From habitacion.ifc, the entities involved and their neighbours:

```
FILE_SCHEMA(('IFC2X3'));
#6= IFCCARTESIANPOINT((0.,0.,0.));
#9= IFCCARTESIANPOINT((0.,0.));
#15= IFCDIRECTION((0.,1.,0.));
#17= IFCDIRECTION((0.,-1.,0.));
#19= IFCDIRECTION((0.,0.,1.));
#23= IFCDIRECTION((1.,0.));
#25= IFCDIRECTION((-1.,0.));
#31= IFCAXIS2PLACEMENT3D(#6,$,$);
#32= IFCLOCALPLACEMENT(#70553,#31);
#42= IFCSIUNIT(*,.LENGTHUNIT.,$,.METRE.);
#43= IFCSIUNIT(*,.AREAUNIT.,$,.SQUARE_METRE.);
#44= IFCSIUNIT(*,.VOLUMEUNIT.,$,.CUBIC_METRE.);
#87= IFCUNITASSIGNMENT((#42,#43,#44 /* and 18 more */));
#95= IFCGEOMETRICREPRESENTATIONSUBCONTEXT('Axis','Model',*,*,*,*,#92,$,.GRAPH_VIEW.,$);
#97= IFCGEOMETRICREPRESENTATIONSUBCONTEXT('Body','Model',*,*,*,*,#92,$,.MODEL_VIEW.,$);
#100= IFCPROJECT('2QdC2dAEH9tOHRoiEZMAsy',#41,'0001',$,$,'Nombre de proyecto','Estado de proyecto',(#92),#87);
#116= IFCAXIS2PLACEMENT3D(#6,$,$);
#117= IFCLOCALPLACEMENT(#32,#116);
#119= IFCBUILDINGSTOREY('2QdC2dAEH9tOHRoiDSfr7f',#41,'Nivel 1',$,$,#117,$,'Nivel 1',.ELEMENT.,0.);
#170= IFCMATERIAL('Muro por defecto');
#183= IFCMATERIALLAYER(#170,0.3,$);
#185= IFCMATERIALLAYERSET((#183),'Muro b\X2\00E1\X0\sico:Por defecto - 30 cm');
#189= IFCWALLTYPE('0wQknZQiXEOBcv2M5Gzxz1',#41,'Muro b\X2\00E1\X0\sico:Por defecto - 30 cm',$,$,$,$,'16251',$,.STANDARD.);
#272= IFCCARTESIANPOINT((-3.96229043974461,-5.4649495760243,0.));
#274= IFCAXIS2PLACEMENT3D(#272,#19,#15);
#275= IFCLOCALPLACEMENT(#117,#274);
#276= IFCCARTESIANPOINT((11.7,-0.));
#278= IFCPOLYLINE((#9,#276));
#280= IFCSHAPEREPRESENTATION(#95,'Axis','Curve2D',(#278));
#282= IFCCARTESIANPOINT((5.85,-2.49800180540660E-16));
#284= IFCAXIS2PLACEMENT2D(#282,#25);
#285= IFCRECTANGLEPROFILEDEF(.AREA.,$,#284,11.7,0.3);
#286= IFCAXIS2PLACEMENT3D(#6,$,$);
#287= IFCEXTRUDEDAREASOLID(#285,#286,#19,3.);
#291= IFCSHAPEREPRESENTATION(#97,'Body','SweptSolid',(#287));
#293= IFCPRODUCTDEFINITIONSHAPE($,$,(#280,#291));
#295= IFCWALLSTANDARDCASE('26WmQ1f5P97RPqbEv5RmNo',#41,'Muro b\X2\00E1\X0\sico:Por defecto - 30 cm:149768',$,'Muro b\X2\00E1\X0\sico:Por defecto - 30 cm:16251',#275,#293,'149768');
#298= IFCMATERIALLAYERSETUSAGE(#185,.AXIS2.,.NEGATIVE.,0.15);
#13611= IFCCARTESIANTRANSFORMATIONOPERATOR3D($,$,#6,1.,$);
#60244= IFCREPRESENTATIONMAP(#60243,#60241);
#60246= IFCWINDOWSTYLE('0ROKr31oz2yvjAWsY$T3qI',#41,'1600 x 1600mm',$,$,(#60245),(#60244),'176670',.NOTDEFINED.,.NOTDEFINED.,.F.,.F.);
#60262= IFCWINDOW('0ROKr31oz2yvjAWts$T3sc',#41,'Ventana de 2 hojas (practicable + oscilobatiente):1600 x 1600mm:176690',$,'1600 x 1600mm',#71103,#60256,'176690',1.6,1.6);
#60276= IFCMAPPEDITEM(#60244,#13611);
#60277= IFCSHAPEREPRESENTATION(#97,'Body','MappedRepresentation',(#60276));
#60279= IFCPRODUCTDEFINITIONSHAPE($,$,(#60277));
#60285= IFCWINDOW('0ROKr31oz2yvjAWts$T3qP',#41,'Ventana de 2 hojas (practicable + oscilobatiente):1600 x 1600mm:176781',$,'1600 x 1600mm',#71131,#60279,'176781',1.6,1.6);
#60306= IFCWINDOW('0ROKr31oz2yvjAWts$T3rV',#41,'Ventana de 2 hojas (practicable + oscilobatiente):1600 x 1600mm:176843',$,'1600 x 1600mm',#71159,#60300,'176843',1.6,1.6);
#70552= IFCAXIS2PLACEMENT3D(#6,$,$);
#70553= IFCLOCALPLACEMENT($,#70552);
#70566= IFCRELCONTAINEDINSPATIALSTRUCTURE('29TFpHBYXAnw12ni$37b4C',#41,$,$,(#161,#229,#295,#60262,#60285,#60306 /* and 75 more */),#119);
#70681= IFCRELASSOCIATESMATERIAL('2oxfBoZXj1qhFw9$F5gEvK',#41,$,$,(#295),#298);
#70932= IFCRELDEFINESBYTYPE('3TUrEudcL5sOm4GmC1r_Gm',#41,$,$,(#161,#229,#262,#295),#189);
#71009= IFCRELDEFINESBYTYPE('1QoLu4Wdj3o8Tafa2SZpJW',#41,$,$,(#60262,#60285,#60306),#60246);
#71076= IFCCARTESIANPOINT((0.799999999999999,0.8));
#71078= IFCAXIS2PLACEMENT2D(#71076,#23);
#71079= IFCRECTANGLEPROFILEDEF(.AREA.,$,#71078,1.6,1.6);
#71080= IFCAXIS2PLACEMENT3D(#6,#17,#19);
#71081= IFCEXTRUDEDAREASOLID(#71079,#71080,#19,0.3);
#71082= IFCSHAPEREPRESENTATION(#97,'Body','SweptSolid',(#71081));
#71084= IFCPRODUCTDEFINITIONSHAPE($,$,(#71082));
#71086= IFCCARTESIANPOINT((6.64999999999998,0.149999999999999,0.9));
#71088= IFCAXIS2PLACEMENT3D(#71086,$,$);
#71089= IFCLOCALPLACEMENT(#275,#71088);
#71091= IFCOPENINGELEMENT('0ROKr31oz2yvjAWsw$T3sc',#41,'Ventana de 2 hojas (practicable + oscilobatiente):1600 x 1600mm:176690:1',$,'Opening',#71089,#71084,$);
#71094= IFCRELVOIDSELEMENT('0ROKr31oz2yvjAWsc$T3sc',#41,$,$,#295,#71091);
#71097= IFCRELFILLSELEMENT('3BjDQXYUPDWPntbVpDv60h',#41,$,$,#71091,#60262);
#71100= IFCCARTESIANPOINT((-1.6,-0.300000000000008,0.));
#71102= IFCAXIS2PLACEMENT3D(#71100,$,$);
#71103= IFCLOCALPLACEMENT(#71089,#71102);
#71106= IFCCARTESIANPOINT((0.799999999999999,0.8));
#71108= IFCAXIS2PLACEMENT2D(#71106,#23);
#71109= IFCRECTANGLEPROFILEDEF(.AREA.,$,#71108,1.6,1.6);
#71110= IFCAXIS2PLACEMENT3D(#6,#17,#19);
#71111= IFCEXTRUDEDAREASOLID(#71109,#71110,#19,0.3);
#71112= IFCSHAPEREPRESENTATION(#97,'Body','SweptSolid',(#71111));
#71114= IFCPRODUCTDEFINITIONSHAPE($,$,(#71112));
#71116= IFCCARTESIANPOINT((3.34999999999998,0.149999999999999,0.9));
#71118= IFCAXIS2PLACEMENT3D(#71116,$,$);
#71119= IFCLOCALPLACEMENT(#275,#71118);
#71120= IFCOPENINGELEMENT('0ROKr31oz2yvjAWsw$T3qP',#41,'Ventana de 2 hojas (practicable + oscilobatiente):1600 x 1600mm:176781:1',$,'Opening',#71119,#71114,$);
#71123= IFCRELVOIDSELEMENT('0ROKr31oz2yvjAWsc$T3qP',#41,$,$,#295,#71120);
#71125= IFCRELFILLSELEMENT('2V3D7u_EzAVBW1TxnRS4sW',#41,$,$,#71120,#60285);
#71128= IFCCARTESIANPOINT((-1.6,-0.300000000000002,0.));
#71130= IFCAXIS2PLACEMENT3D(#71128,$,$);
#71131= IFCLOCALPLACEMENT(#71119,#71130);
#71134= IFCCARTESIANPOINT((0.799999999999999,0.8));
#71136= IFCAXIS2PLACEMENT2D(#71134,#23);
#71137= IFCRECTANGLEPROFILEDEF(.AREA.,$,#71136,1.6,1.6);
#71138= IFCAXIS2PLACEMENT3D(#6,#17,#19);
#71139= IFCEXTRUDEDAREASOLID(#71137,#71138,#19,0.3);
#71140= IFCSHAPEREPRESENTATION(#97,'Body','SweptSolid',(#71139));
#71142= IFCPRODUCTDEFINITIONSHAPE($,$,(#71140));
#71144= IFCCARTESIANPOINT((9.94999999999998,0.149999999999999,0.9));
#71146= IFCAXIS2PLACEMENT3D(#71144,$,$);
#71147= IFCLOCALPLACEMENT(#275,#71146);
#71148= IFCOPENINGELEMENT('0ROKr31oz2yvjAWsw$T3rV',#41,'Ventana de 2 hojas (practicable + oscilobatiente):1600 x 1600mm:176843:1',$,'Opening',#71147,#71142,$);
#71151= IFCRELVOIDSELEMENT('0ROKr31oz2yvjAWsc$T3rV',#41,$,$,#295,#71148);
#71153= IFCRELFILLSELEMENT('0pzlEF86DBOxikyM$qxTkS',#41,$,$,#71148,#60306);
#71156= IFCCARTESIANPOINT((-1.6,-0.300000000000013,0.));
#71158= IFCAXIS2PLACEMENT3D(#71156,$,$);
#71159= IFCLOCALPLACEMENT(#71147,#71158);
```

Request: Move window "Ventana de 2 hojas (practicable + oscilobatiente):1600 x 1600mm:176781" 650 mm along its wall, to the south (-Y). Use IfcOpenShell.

```python
import ifcopenshell
import ifcopenshell.api.geometry
import ifcopenshell.util.placement

model = ifcopenshell.open("habitacion.ifc")

window = model.by_guid("0ROKr31oz2yvjAWts$T3qP")
opening = window.FillsVoids[0].RelatingOpeningElement
wall = opening.VoidsElements[0].RelatingBuildingElement

wall_matrix = ifcopenshell.util.placement.get_local_placement(wall.ObjectPlacement)
shift = wall_matrix[:3, 0] * -0.65
before = ifcopenshell.util.placement.get_local_placement(window.ObjectPlacement)[:3, 3].copy()

# The window is placed relative to its opening, so it follows when the opening moves.
matrix = ifcopenshell.util.placement.get_local_placement(opening.ObjectPlacement)
matrix[:3, 3] += shift
ifcopenshell.api.geometry.edit_object_placement(
    model, product=opening, matrix=matrix, is_si=False, should_transform_children=True
)

after = ifcopenshell.util.placement.get_local_placement(window.ObjectPlacement)[:3, 3]
print("window moved by", (after - before).round(3) + 0.0)

model.write("habitacion_rev.ifc")
```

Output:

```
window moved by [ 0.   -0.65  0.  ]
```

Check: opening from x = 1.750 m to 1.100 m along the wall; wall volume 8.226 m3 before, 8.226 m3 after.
